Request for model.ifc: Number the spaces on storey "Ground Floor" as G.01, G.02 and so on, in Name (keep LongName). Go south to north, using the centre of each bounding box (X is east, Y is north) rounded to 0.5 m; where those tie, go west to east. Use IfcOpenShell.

First a look at what the model holds.

```python
import ifcopenshell
import ifcopenshell.util.element
import ifcopenshell.util.placement

model = ifcopenshell.open("model.ifc")
print(model.schema)
storey = next(s for s in model.by_type("IfcBuildingStorey") if s.Name == "Ground Floor")
spaces = [e for e in ifcopenshell.util.element.get_decomposition(storey) if e.is_a("IfcSpace")]
for e in sorted(spaces, key=lambda e: e.id()):
    origin = ifcopenshell.util.placement.get_local_placement(e.ObjectPlacement)[:3, 3]
    print(e.id(), e.Name, e.LongName, origin.round(2) + 0.0, sep=" | ")
```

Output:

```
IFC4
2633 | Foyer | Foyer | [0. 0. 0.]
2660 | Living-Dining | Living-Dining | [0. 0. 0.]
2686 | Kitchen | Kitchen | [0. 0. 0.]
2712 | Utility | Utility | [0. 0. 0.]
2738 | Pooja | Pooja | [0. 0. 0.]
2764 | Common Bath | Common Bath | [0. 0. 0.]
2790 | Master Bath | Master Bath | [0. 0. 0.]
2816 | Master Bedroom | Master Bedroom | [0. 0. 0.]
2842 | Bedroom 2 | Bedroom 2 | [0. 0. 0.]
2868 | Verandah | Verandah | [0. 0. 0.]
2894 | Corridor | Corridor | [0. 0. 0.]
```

```python
import ifcopenshell
import ifcopenshell.geom
import ifcopenshell.util.element
import ifcopenshell.util.shape

model = ifcopenshell.open("model.ifc")
settings = ifcopenshell.geom.settings()
settings.set("use-world-coords", True)


def centre(element):
    shape = ifcopenshell.geom.create_shape(settings, element)
    return ifcopenshell.util.shape.get_bbox_centroid(shape.geometry)


storey = next(s for s in model.by_type("IfcBuildingStorey") if s.Name == "Ground Floor")
spaces = [e for e in ifcopenshell.util.element.get_decomposition(storey) if e.is_a("IfcSpace")]

# Insertion points can sit at a corner or the storey origin, so sort by the geometry (in metres).
centres = {e: centre(e) for e in spaces}
spaces.sort(key=lambda e: (round(centres[e][1] / 0.5), centres[e][0]))

for i, e in enumerate(spaces, start=1):
    number = f"G.{i:02d}"
    e.Name = number
    print(e.id(), number)

model.write("model_rev.ifc")
```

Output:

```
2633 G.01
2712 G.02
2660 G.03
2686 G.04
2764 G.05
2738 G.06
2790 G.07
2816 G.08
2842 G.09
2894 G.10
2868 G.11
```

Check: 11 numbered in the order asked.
